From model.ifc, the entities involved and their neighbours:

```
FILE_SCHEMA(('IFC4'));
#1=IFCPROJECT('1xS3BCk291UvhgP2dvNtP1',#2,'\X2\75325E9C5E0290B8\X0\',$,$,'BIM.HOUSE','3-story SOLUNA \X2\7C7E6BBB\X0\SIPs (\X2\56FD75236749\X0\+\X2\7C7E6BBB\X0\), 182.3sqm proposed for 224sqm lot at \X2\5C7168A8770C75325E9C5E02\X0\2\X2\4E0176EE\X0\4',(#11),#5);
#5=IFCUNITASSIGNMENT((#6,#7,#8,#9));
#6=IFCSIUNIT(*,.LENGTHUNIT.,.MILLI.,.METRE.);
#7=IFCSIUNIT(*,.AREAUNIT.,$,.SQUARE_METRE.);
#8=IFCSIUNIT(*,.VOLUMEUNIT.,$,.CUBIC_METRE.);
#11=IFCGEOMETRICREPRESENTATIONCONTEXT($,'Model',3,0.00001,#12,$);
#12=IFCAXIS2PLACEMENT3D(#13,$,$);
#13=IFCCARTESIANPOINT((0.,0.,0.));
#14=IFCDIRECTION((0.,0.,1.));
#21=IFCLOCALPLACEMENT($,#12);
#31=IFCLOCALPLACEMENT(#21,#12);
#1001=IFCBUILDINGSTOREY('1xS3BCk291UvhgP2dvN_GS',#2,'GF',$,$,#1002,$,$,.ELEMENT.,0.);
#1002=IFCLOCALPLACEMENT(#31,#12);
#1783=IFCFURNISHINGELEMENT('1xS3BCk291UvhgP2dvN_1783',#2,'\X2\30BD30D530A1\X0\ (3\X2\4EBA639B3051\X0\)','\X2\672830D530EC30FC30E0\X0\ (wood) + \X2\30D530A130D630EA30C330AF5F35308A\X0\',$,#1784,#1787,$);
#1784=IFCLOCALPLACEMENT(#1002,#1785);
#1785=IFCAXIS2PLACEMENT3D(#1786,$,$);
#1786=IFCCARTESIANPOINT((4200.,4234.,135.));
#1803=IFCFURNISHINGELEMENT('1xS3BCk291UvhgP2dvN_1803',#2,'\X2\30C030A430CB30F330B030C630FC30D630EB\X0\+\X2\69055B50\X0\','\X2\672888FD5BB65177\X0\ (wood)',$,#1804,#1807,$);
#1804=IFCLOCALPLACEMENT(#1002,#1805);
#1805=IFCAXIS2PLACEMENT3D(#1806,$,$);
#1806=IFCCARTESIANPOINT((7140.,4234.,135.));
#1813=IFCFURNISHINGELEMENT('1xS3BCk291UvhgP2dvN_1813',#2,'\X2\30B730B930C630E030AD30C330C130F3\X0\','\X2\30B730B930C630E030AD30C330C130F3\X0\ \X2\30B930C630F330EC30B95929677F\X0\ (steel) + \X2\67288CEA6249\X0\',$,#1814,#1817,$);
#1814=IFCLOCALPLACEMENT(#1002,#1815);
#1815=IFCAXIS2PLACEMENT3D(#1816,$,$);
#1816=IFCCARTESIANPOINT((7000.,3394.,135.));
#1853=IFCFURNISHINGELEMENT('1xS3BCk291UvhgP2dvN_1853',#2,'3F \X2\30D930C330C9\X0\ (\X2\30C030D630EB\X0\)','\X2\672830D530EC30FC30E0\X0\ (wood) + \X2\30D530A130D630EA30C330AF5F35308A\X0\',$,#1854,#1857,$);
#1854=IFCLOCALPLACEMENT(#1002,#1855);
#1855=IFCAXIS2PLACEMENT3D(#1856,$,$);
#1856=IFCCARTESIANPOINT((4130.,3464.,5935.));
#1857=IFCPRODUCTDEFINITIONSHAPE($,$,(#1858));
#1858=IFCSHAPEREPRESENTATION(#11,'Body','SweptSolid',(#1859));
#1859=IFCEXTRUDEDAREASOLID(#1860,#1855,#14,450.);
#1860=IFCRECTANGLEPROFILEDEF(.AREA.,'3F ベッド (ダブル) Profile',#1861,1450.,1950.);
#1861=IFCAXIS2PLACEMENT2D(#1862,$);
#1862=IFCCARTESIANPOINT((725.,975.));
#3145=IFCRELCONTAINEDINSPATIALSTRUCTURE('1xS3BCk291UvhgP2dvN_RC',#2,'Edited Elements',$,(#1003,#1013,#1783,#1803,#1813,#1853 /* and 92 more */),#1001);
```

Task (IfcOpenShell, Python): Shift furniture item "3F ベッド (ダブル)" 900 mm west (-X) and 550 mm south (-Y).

```python
import ifcopenshell
import ifcopenshell.api.geometry
import ifcopenshell.util.placement

model = ifcopenshell.open("model.ifc")

item = model.by_guid("1xS3BCk291UvhgP2dvN_1853")
matrix = ifcopenshell.util.placement.get_local_placement(item.ObjectPlacement)
matrix[0, 3] -= 900.0
matrix[1, 3] -= 550.0
ifcopenshell.api.geometry.edit_object_placement(model, product=item, matrix=matrix, is_si=False)

print(ifcopenshell.util.placement.get_local_placement(item.ObjectPlacement).round(3) + 0.0)

model.write("model_rev.ifc")
```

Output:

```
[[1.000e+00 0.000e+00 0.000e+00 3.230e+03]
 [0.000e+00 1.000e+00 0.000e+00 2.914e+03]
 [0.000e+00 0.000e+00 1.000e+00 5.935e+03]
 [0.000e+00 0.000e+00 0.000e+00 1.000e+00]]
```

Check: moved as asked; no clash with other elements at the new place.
